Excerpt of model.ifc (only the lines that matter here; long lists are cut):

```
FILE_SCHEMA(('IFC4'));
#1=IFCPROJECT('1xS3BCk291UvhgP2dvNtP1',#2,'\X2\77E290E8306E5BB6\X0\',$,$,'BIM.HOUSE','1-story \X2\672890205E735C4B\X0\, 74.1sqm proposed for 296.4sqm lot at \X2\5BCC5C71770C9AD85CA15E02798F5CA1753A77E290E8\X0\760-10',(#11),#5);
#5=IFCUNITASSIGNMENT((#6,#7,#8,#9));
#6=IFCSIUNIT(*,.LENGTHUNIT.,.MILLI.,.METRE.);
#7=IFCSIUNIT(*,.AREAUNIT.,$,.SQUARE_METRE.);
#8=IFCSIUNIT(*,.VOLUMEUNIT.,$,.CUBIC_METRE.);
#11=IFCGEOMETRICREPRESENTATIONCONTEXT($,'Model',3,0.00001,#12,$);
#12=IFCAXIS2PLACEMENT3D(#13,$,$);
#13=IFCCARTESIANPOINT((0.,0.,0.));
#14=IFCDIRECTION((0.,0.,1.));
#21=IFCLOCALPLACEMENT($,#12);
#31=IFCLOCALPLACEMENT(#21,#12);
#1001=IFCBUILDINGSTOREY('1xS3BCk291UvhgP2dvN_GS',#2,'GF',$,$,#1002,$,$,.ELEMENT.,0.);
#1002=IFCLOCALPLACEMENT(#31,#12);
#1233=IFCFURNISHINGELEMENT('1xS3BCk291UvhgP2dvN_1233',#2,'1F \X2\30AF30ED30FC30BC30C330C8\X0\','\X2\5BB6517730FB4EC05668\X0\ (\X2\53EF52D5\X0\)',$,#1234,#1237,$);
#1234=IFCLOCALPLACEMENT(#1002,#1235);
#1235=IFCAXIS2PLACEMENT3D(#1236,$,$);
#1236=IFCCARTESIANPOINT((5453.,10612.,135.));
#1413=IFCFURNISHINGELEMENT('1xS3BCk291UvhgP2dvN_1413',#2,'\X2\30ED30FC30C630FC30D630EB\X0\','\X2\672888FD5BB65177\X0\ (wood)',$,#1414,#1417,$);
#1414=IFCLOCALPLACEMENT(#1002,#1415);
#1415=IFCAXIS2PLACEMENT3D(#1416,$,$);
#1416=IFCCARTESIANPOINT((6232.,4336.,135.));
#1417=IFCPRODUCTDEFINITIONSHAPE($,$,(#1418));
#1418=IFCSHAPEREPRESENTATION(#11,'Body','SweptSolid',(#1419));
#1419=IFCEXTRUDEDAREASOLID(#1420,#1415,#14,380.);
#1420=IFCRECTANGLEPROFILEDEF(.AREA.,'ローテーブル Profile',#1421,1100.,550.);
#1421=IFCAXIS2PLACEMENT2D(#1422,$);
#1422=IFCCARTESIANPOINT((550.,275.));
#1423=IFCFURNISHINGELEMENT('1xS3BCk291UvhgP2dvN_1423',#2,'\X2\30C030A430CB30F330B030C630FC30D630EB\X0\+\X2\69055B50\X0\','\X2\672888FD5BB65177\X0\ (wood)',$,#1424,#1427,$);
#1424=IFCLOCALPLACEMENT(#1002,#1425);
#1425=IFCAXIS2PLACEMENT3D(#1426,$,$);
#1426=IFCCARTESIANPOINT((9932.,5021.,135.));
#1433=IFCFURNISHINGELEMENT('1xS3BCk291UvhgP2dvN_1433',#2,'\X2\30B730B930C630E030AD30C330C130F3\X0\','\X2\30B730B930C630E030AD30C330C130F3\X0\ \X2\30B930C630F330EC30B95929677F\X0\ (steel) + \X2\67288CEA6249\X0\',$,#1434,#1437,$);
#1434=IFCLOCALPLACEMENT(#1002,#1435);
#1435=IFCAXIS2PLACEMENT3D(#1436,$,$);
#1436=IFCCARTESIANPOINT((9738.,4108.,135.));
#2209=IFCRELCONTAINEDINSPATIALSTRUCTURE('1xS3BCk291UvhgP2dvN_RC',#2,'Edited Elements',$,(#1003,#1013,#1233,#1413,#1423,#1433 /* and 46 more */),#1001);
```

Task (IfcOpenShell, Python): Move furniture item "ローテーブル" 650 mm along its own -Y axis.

```python
import ifcopenshell
import ifcopenshell.api.geometry
import ifcopenshell.util.placement
import ifcopenshell.util.unit

model = ifcopenshell.open("model.ifc")
unit_scale = ifcopenshell.util.unit.calculate_unit_scale(model)

item = model.by_id(1413)
matrix = ifcopenshell.util.placement.get_local_placement(item.ObjectPlacement)
matrix[:3, 3] -= matrix[:3, 1] * 0.65 / unit_scale
ifcopenshell.api.geometry.edit_object_placement(model, product=item, matrix=matrix, is_si=False)

print(ifcopenshell.util.placement.get_local_placement(item.ObjectPlacement).round(3) + 0.0)

model.write("model-out.ifc")
```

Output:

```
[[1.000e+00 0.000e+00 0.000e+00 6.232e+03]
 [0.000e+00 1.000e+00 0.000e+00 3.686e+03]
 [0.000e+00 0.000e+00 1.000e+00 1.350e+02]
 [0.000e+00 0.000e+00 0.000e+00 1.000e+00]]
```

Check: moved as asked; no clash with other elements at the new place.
